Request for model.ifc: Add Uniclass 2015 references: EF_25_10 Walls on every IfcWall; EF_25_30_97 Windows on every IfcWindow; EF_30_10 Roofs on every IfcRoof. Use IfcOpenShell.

First a look at what the model holds.

```python
import ifcopenshell

model = ifcopenshell.open("model.ifc")
print(model.schema)
print("classifications:", [c.Name for c in model.by_type("IfcClassification")])
for ifc_class in ("IfcDoor", "IfcRoof", "IfcStair", "IfcWall", "IfcWindow"):
    print(ifc_class, len(model.by_type(ifc_class)))
```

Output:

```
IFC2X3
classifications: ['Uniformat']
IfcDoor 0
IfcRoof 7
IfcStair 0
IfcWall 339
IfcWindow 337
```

```python
import ifcopenshell
import ifcopenshell.api.classification

model = ifcopenshell.open("model.ifc")

# IFC2X3 requires Source and Edition and has no link from the project to the system.
system = model.create_entity("IfcClassification", Source="NBS", Edition="2015", Name="Uniclass 2015")

codes = {
    "IfcWall": ("EF_25_10", "Walls"),
    "IfcWindow": ("EF_25_30_97", "Windows"),
    "IfcRoof": ("EF_30_10", "Roofs"),
}
for ifc_class, (code, name) in codes.items():
    products = model.by_type(ifc_class)
    ifcopenshell.api.classification.add_reference(
        model, products=products, classification=system, identification=code, name=name
    )
    print(code, len(products))

model.write("model_rev.ifc")
```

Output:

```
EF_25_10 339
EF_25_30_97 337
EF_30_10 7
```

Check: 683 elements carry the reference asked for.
